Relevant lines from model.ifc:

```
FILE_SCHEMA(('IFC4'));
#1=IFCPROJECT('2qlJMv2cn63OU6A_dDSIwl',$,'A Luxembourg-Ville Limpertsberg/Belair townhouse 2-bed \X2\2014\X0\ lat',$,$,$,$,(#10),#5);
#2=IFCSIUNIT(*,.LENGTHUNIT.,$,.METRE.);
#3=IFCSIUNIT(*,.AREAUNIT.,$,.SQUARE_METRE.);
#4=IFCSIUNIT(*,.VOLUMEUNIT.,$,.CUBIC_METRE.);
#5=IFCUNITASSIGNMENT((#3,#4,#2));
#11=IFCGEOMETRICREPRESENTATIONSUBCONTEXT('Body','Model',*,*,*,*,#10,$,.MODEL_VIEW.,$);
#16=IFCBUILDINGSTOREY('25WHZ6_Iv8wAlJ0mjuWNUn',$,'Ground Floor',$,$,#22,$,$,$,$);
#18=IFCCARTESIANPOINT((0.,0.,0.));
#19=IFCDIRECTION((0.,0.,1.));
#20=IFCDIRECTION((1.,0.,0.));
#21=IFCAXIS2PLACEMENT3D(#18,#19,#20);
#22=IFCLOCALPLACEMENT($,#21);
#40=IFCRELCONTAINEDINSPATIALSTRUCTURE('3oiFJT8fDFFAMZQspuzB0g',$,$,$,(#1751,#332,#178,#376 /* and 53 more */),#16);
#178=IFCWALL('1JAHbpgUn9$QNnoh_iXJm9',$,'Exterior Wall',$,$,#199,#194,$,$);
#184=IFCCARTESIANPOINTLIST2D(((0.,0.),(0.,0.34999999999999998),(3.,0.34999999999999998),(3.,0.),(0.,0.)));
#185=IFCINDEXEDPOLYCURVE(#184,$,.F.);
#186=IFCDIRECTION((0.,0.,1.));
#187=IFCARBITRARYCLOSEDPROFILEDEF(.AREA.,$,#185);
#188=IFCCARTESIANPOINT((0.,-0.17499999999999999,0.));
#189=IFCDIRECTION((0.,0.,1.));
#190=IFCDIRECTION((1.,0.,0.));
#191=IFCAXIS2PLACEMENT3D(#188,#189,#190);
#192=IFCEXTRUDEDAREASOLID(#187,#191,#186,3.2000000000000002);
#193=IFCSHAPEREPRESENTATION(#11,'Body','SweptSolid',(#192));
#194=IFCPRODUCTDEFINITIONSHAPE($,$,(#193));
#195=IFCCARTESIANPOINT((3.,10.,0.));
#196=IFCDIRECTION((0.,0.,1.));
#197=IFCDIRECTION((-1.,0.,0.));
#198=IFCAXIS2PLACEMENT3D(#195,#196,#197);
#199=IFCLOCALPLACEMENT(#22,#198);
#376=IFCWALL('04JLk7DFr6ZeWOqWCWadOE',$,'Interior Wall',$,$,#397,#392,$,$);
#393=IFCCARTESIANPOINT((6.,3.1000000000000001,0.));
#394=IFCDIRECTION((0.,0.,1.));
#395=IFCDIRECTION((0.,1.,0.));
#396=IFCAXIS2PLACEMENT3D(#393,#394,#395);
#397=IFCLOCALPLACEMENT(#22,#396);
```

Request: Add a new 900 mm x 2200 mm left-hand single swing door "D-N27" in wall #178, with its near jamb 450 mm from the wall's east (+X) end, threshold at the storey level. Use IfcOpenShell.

```python
import numpy as np
import ifcopenshell
import ifcopenshell.api.feature
import ifcopenshell.api.geometry
import ifcopenshell.api.root
import ifcopenshell.api.spatial
import ifcopenshell.geom
import ifcopenshell.util.element
import ifcopenshell.util.placement
import ifcopenshell.util.representation
import ifcopenshell.util.shape
import ifcopenshell.util.unit

model = ifcopenshell.open("model.ifc")
unit_scale = ifcopenshell.util.unit.calculate_unit_scale(model)
settings = ifcopenshell.geom.settings()


def volume(element):
    """Net volume in cubic metres, openings subtracted."""
    shape = ifcopenshell.geom.create_shape(settings, element)
    return ifcopenshell.util.shape.get_volume(shape.geometry)


wall = model.by_guid("1JAHbpgUn9$QNnoh_iXJm9")
storey = ifcopenshell.util.element.get_container(wall, ifc_class="IfcBuildingStorey")
context = ifcopenshell.util.representation.get_context(model, "Model", "Body", "MODEL_VIEW")
before = volume(wall)

width, height, from_end, sill = 0.9, 2.2, 0.45, 0.0  # metres

# The wall runs along its own X axis, and the end named is its -X end.
wall_shape = ifcopenshell.geom.create_shape(settings, wall)
x, y, z = ifcopenshell.util.shape.get_vertices(wall_shape.geometry).T
start = x.min() + from_end
face, thickness = float(y.min()), float(y.max() - y.min())
wall_matrix = ifcopenshell.util.placement.get_local_placement(wall.ObjectPlacement)
level = ifcopenshell.util.placement.get_local_placement(storey.ObjectPlacement)[2, 3]


def in_wall(x, y):
    """Placement at x, y metres in the wall's axes, at sill height."""
    matrix = wall_matrix.copy()
    matrix[:, 3] = wall_matrix @ np.array([x / unit_scale, y / unit_scale, 0.0, 1.0])
    matrix[2, 3] = level + sill / unit_scale
    return matrix


# Opening: a box that overshoots both wall faces by 50 mm.
opening = ifcopenshell.api.root.create_entity(model, ifc_class="IfcOpeningElement", predefined_type="OPENING")
box = ifcopenshell.api.geometry.add_wall_representation(
    model, context=context, length=width, height=height, thickness=thickness + 0.1
)
ifcopenshell.api.geometry.assign_representation(model, product=opening, representation=box)
ifcopenshell.api.geometry.edit_object_placement(model, product=opening, matrix=in_wall(start, face - 0.05), is_si=False)
ifcopenshell.api.feature.add_feature(model, feature=opening, element=wall)

door = ifcopenshell.api.root.create_entity(model, ifc_class="IfcDoor", name="D-N27", predefined_type="DOOR")
door.OverallWidth, door.OverallHeight = width / unit_scale, height / unit_scale
door.OperationType = "SINGLE_SWING_LEFT"
body = ifcopenshell.api.geometry.add_door_representation(
    model,
    context=context,
    overall_width=door.OverallWidth,
    overall_height=door.OverallHeight,
    operation_type="SINGLE_SWING_LEFT",
    lining_properties={"LiningDepth": thickness / unit_scale, "ThresholdDepth": thickness / unit_scale},
)
ifcopenshell.api.geometry.assign_representation(model, product=door, representation=body)
ifcopenshell.api.spatial.assign_container(model, products=[door], relating_structure=storey)
ifcopenshell.api.feature.add_filling(model, opening=opening, element=door)

# The lining spans the wall, so the door starts at the wall face.
ifcopenshell.api.geometry.edit_object_placement(model, product=door, matrix=in_wall(start, face), is_si=False)

after = volume(wall)

print(f"wall volume {before:.3f} -> {after:.3f} m3")

model.write("model_v2.ifc")
```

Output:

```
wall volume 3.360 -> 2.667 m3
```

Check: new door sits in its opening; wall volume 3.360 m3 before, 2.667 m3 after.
